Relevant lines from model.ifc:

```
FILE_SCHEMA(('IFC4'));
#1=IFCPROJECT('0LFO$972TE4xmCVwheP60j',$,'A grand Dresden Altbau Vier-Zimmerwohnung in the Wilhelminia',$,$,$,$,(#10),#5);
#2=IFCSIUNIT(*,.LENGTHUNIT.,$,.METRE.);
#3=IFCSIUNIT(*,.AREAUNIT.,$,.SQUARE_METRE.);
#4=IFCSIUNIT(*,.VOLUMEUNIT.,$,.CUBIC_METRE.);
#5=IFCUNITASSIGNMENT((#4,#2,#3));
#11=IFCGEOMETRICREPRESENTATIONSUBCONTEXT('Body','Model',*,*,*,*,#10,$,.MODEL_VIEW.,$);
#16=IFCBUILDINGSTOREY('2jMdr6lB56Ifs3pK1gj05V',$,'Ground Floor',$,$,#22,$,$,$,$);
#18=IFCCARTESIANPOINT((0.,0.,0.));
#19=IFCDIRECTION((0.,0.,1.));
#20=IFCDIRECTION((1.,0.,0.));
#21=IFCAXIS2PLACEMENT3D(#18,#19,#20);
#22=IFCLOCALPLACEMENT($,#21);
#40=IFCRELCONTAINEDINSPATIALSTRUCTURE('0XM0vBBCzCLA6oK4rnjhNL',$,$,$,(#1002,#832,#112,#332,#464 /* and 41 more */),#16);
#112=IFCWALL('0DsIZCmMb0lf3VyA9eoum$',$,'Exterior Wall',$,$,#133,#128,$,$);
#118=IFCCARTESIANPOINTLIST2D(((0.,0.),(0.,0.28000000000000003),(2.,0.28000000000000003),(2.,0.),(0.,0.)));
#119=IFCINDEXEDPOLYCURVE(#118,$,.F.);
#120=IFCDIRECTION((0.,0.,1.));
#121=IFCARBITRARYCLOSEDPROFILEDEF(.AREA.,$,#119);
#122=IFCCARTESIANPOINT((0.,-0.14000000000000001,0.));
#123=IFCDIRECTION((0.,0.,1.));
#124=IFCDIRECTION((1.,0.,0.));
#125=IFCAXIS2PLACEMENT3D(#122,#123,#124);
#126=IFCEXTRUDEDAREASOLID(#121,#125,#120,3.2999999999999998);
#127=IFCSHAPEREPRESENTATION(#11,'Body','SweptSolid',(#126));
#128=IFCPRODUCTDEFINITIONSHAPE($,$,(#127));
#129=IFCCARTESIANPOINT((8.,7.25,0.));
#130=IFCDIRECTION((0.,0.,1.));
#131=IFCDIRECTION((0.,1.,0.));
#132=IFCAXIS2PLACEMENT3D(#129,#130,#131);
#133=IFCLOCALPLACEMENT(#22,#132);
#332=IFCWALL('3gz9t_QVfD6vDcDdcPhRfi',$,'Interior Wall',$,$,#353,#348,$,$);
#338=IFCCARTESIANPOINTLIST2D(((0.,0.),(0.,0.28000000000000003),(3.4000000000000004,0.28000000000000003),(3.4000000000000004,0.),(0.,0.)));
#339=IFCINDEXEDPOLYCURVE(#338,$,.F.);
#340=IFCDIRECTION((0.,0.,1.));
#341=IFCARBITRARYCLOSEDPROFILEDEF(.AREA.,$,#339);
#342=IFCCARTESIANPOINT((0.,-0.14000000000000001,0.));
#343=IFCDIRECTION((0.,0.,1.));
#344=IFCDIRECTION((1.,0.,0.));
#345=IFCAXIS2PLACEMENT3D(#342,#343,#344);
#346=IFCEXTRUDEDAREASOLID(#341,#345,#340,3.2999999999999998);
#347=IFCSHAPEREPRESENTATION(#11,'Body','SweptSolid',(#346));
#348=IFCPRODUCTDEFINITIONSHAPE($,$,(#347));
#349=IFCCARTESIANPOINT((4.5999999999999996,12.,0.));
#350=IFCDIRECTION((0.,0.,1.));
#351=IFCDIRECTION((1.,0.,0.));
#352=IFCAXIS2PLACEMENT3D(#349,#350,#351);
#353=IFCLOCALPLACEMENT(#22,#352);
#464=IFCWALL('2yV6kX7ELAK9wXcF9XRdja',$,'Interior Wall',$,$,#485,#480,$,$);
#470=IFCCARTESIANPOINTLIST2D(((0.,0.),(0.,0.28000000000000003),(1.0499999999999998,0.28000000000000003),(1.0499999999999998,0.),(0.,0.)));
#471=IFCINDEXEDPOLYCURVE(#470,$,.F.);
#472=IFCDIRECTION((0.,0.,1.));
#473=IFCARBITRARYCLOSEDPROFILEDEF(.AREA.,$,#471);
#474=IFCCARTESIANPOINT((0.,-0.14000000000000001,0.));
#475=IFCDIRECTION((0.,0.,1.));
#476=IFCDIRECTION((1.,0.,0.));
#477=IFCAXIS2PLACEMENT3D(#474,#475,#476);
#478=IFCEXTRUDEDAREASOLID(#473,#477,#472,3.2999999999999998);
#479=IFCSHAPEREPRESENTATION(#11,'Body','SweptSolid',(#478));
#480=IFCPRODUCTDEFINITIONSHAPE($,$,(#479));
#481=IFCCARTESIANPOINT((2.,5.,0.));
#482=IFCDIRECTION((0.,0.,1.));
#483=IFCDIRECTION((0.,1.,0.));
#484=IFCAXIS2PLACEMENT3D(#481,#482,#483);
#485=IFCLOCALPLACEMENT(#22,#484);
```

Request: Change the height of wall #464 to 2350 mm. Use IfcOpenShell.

```python
import ifcopenshell
import ifcopenshell.geom
import ifcopenshell.util.representation
import ifcopenshell.util.shape
import ifcopenshell.util.unit

model = ifcopenshell.open("model.ifc")
unit_scale = ifcopenshell.util.unit.calculate_unit_scale(model)
settings = ifcopenshell.geom.settings()


def volume(element):
    """Net volume in cubic metres, openings subtracted."""
    shape = ifcopenshell.geom.create_shape(settings, element)
    return ifcopenshell.util.shape.get_volume(shape.geometry)


wall = model.by_guid("2yV6kX7ELAK9wXcF9XRdja")
before = volume(wall)

body = ifcopenshell.util.representation.get_representation(wall, "Model", "Body")
solid = body.Items[0]
old_height = solid.Depth
solid.Depth = 2.35 / unit_scale
after = volume(wall)

print(f"height {old_height:g} -> {solid.Depth:g}, volume {before:.3f} -> {after:.3f} m3")

model.write("model-out.ifc")
```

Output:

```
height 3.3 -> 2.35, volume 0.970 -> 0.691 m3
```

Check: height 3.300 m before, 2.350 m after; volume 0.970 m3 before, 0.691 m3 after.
